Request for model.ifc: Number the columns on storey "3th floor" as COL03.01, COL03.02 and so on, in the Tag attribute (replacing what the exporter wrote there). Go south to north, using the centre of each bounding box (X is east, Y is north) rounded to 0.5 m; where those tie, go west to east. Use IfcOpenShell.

First a look at what the model holds.

```python
import ifcopenshell
import ifcopenshell.util.element
import ifcopenshell.util.placement

model = ifcopenshell.open("model.ifc")
print(model.schema)
storey = next(s for s in model.by_type("IfcBuildingStorey") if s.Name == "3th floor")
columns = [e for e in ifcopenshell.util.element.get_decomposition(storey) if e.is_a("IfcColumn")]
for e in sorted(columns, key=lambda e: e.id()):
    origin = ifcopenshell.util.placement.get_local_placement(e.ObjectPlacement)[:3, 3]
    print(e.id(), e.Tag, e.Name, origin.round(2) + 0.0, sep=" | ")
```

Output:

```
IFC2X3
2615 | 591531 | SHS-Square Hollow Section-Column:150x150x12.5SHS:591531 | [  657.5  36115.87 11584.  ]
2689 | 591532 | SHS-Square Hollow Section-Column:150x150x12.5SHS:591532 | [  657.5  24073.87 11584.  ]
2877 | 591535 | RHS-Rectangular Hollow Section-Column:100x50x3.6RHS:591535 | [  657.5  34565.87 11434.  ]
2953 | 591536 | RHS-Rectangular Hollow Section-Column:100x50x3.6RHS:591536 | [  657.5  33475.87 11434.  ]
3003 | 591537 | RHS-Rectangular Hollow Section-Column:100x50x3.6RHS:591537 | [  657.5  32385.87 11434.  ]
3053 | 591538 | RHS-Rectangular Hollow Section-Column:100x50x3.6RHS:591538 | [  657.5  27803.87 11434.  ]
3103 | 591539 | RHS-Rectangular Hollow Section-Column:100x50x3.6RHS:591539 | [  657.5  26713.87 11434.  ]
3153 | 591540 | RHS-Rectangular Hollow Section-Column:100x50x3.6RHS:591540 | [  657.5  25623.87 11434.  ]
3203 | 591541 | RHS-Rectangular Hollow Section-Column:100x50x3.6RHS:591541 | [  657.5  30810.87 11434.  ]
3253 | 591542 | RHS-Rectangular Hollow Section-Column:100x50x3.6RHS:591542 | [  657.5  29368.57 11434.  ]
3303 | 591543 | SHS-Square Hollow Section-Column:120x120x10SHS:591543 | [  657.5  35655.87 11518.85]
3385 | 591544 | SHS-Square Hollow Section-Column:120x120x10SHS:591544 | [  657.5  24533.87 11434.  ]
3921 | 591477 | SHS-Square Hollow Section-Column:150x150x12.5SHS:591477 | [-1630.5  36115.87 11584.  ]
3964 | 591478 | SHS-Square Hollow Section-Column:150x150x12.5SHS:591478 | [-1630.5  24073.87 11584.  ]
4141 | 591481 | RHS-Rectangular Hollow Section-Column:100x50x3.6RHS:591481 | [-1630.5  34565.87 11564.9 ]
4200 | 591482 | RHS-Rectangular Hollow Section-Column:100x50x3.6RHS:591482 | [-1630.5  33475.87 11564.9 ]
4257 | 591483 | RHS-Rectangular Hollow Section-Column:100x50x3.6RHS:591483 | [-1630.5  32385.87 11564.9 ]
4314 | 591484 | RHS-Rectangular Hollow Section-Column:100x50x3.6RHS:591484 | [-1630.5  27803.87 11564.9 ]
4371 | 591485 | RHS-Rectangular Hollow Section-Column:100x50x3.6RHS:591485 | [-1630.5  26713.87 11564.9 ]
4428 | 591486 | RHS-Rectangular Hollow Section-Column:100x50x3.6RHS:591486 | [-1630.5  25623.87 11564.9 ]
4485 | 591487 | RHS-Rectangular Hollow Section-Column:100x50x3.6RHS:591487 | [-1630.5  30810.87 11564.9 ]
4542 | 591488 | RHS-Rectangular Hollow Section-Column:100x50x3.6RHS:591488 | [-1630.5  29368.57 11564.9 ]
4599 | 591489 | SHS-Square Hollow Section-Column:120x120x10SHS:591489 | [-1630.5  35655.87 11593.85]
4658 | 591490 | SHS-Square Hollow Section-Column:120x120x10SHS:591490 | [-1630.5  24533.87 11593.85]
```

```python
import ifcopenshell
import ifcopenshell.geom
import ifcopenshell.util.element
import ifcopenshell.util.shape

model = ifcopenshell.open("model.ifc")
settings = ifcopenshell.geom.settings()
settings.set("use-world-coords", True)


def centre(element):
    shape = ifcopenshell.geom.create_shape(settings, element)
    return ifcopenshell.util.shape.get_bbox_centroid(shape.geometry)


storey = next(s for s in model.by_type("IfcBuildingStorey") if s.Name == "3th floor")
columns = [e for e in ifcopenshell.util.element.get_decomposition(storey) if e.is_a("IfcColumn")]

# Insertion points can sit at a corner or the storey origin, so sort by the geometry (in metres).
centres = {e: centre(e) for e in columns}
columns.sort(key=lambda e: (round(centres[e][1] / 0.5), centres[e][0]))

for i, e in enumerate(columns, start=1):
    number = f"COL03.{i:02d}"
    e.Tag = number
    print(e.id(), number)

model.write("model_updated.ifc")
```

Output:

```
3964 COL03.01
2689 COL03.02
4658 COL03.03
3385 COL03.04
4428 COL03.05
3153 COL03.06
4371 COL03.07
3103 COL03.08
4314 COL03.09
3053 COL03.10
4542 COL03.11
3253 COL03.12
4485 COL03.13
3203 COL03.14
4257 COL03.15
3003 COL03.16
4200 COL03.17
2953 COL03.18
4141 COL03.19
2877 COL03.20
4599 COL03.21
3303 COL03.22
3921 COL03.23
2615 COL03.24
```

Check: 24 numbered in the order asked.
